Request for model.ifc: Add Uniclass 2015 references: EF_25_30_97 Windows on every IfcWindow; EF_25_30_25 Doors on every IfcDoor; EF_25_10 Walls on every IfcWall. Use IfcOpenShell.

First a look at what the model holds.

```python
import ifcopenshell

model = ifcopenshell.open("model.ifc")
print(model.schema)
print("classifications:", [c.Name for c in model.by_type("IfcClassification")])
for ifc_class in ("IfcDoor", "IfcRoof", "IfcStair", "IfcWall", "IfcWindow"):
    print(ifc_class, len(model.by_type(ifc_class)))
```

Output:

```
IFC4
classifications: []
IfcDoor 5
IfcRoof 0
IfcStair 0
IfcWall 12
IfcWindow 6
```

```python
import ifcopenshell
import ifcopenshell.api.classification

model = ifcopenshell.open("model.ifc")

system = ifcopenshell.api.classification.add_classification(model, classification="Uniclass 2015")

codes = {
    "IfcWindow": ("EF_25_30_97", "Windows"),
    "IfcDoor": ("EF_25_30_25", "Doors"),
    "IfcWall": ("EF_25_10", "Walls"),
}
for ifc_class, (code, name) in codes.items():
    products = model.by_type(ifc_class)
    ifcopenshell.api.classification.add_reference(
        model, products=products, classification=system, identification=code, name=name
    )
    print(code, len(products))

model.write("model_edited.ifc")
```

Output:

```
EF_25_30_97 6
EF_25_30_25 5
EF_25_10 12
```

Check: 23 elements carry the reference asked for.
